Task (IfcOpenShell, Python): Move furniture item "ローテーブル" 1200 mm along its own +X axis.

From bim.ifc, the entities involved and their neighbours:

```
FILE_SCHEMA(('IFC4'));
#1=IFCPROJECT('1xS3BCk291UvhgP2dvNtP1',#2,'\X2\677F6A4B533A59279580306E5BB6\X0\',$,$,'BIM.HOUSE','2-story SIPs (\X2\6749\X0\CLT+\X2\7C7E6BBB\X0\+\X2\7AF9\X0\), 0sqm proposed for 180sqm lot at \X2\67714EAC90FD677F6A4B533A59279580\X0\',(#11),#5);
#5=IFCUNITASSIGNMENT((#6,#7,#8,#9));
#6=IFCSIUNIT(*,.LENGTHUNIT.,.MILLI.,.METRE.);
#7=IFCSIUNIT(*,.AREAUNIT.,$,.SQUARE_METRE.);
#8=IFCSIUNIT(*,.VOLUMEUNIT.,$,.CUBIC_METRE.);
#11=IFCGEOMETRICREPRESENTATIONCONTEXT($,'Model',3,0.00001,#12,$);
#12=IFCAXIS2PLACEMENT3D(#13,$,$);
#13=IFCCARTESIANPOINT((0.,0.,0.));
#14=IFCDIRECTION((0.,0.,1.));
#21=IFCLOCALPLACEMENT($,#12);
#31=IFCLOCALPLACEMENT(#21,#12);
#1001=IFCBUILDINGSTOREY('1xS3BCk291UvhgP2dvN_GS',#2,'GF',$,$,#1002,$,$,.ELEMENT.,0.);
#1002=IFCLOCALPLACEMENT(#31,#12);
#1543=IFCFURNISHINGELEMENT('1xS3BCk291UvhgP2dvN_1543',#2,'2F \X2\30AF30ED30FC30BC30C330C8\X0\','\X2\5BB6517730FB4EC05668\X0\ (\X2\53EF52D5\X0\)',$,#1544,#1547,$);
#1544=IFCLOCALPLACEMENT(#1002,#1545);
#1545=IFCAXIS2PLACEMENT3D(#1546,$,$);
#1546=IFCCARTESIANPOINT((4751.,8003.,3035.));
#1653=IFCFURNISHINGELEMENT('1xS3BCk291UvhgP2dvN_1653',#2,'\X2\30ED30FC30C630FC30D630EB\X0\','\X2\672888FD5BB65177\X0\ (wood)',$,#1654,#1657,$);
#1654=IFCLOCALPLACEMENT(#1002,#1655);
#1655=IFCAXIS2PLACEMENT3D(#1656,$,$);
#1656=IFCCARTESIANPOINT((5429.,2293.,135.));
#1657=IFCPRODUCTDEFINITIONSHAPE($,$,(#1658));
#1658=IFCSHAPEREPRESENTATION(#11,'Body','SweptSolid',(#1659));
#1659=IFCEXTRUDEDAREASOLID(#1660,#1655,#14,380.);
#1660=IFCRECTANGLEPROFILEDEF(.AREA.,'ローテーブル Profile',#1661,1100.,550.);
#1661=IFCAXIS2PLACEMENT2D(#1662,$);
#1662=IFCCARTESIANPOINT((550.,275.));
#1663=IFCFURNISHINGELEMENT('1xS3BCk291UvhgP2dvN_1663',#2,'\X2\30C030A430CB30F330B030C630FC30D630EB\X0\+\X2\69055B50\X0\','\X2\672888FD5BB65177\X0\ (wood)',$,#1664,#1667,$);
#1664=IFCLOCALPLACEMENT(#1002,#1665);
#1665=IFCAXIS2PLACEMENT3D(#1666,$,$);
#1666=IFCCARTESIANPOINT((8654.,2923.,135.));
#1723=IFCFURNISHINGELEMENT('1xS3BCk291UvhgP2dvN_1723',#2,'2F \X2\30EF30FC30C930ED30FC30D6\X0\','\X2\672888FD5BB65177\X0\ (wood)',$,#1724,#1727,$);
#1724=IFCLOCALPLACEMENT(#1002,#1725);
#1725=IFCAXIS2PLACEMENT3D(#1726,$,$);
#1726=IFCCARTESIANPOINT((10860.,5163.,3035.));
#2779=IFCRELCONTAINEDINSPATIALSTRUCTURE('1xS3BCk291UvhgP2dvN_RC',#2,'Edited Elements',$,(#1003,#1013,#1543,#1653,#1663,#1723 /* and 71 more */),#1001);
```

```python
import ifcopenshell
import ifcopenshell.api.geometry
import ifcopenshell.util.placement
import ifcopenshell.util.unit

model = ifcopenshell.open("bim.ifc")
unit_scale = ifcopenshell.util.unit.calculate_unit_scale(model)

item = model.by_id(1653)
matrix = ifcopenshell.util.placement.get_local_placement(item.ObjectPlacement)
matrix[:3, 3] += matrix[:3, 0] * 1.2 / unit_scale
ifcopenshell.api.geometry.edit_object_placement(model, product=item, matrix=matrix, is_si=False)

print(ifcopenshell.util.placement.get_local_placement(item.ObjectPlacement).round(3) + 0.0)

model.write("bim_updated.ifc")
```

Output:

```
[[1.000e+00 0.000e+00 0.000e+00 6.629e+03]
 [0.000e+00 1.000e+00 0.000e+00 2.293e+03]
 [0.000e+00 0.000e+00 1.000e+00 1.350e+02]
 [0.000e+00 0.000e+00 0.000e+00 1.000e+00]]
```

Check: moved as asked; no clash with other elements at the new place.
